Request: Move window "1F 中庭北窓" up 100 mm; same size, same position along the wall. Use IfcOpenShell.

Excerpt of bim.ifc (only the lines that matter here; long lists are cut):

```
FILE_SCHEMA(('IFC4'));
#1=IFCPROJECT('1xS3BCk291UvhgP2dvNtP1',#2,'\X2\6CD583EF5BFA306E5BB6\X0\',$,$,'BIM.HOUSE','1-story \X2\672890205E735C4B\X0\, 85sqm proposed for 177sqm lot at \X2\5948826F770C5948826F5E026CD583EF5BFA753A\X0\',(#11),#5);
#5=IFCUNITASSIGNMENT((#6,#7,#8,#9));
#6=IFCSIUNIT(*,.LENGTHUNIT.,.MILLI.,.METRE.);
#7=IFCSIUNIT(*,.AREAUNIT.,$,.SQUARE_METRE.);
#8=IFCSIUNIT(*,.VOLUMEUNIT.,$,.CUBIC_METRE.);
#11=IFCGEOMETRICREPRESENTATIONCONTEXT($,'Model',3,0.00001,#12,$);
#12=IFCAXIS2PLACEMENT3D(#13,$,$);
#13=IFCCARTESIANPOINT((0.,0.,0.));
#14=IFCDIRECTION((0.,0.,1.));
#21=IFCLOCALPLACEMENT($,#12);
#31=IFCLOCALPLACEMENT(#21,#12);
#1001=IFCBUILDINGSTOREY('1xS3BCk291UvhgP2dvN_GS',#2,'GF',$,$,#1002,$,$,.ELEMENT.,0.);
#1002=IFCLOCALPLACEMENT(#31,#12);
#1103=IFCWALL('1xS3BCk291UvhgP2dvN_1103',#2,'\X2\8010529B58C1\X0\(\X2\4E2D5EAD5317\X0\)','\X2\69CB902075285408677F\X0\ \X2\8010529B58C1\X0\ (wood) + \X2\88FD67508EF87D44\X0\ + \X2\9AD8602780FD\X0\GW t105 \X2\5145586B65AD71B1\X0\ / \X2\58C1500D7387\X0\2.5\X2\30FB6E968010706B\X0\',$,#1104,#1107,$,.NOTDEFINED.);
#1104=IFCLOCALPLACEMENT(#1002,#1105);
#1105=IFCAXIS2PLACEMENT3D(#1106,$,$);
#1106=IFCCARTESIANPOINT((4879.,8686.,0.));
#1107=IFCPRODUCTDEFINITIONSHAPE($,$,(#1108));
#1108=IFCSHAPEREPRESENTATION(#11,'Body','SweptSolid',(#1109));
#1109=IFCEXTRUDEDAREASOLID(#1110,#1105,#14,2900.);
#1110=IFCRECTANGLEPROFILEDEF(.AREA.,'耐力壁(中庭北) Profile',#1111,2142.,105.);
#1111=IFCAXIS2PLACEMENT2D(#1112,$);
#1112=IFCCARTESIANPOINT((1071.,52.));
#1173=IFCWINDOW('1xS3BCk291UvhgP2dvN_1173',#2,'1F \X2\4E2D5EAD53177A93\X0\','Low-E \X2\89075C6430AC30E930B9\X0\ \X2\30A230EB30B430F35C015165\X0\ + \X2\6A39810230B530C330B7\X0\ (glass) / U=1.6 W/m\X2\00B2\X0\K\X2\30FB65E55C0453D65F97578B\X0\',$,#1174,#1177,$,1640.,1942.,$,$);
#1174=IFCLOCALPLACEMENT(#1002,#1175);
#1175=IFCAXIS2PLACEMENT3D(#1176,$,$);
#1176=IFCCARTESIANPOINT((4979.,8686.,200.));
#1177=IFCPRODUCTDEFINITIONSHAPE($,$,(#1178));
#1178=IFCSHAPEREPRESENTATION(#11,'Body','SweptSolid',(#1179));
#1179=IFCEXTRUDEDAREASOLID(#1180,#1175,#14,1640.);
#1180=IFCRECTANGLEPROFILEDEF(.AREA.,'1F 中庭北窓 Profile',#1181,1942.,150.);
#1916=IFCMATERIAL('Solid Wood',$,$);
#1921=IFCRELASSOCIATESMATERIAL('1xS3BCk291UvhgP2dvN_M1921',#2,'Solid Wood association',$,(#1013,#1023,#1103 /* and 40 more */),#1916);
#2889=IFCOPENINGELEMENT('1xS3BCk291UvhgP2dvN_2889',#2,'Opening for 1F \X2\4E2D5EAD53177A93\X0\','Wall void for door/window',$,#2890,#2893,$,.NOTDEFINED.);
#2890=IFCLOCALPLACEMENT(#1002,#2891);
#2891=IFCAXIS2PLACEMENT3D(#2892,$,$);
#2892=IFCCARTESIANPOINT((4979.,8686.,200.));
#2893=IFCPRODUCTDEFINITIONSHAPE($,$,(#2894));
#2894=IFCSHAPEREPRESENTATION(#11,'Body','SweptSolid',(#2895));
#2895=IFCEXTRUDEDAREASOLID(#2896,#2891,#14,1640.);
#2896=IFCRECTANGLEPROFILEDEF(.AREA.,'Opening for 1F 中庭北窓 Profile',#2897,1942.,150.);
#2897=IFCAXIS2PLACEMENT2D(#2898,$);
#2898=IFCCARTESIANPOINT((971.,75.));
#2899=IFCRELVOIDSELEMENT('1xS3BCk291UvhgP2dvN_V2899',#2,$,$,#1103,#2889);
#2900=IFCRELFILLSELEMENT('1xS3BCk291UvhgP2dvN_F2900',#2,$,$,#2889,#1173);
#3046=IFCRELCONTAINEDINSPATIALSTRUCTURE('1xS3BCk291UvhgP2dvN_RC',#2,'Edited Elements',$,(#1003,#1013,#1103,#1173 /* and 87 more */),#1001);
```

```python
import numpy as np
import ifcopenshell
import ifcopenshell.api.geometry
import ifcopenshell.util.placement
import ifcopenshell.util.unit

model = ifcopenshell.open("bim.ifc")
unit_scale = ifcopenshell.util.unit.calculate_unit_scale(model)

window = model.by_guid("1xS3BCk291UvhgP2dvN_1173")
opening = window.FillsVoids[0].RelatingOpeningElement
dz = 100.0

shift = np.array([0.0, 0.0, dz])
# The window is not placed relative to its opening, so move both.
for product in (opening, window):
    matrix = ifcopenshell.util.placement.get_local_placement(product.ObjectPlacement)
    matrix[:3, 3] += shift
    ifcopenshell.api.geometry.edit_object_placement(model, product=product, matrix=matrix, is_si=False)

print(f"moved by {dz * unit_scale:+.3f} m")

model.write("bim_v2.ifc")
```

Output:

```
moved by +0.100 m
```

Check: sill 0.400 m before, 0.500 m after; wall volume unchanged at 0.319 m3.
